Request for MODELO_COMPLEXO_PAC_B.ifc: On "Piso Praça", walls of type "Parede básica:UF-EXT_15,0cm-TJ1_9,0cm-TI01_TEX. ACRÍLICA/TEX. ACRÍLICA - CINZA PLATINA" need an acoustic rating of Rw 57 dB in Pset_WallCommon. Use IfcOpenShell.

First a look at what the model holds.

```python
import ifcopenshell
import ifcopenshell.util.element

model = ifcopenshell.open("MODELO_COMPLEXO_PAC_B.ifc")
print(model.schema)
storey = next(s for s in model.by_type("IfcBuildingStorey") if s.Name == "Piso Praça")
walls = [e for e in ifcopenshell.util.element.get_decomposition(storey) if e.is_a("IfcWall")]
seen = {}
for e in walls:
    element_type = ifcopenshell.util.element.get_type(e)
    key = (element_type.Name if element_type != e and element_type else None, ifcopenshell.util.element.get_pset(e, "Pset_WallCommon", "AcousticRating"))
    seen[key] = seen.get(key, 0) + 1
for (name, value), count in sorted(seen.items(), key=str):
    print(count, "x", name, "|", value)
```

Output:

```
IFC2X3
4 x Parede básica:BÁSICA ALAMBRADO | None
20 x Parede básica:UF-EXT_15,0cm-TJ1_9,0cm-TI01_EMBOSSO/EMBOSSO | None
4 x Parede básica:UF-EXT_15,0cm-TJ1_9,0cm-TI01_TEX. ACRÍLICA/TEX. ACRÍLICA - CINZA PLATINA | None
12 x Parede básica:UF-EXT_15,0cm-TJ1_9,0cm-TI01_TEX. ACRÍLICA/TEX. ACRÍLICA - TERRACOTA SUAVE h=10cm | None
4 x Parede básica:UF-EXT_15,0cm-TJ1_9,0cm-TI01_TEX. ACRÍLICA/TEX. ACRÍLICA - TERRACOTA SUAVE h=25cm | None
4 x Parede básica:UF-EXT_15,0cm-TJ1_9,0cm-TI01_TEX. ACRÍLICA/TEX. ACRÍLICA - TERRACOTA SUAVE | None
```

```python
import ifcopenshell
import ifcopenshell.api.pset
import ifcopenshell.util.element

model = ifcopenshell.open("MODELO_COMPLEXO_PAC_B.ifc")

storey = next(s for s in model.by_type("IfcBuildingStorey") if s.Name == "Piso Praça")
walls = [e for e in ifcopenshell.util.element.get_decomposition(storey) if e.is_a("IfcWall")]

count = 0
for e in walls:
    element_type = ifcopenshell.util.element.get_type(e)
    if element_type in (None, e) or element_type.Name != "Parede básica:UF-EXT_15,0cm-TJ1_9,0cm-TI01_TEX. ACRÍLICA/TEX. ACRÍLICA - CINZA PLATINA":
        continue
    # add_pset returns the element's existing set when there is one.
    pset = ifcopenshell.api.pset.add_pset(model, product=e, name="Pset_WallCommon")
    ifcopenshell.api.pset.edit_pset(model, pset=pset, properties={"AcousticRating": "Rw 57 dB"})
    count += 1

print(count, "walls updated")

model.write("MODELO_COMPLEXO_PAC_B-out.ifc")
```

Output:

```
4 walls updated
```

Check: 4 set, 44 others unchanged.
